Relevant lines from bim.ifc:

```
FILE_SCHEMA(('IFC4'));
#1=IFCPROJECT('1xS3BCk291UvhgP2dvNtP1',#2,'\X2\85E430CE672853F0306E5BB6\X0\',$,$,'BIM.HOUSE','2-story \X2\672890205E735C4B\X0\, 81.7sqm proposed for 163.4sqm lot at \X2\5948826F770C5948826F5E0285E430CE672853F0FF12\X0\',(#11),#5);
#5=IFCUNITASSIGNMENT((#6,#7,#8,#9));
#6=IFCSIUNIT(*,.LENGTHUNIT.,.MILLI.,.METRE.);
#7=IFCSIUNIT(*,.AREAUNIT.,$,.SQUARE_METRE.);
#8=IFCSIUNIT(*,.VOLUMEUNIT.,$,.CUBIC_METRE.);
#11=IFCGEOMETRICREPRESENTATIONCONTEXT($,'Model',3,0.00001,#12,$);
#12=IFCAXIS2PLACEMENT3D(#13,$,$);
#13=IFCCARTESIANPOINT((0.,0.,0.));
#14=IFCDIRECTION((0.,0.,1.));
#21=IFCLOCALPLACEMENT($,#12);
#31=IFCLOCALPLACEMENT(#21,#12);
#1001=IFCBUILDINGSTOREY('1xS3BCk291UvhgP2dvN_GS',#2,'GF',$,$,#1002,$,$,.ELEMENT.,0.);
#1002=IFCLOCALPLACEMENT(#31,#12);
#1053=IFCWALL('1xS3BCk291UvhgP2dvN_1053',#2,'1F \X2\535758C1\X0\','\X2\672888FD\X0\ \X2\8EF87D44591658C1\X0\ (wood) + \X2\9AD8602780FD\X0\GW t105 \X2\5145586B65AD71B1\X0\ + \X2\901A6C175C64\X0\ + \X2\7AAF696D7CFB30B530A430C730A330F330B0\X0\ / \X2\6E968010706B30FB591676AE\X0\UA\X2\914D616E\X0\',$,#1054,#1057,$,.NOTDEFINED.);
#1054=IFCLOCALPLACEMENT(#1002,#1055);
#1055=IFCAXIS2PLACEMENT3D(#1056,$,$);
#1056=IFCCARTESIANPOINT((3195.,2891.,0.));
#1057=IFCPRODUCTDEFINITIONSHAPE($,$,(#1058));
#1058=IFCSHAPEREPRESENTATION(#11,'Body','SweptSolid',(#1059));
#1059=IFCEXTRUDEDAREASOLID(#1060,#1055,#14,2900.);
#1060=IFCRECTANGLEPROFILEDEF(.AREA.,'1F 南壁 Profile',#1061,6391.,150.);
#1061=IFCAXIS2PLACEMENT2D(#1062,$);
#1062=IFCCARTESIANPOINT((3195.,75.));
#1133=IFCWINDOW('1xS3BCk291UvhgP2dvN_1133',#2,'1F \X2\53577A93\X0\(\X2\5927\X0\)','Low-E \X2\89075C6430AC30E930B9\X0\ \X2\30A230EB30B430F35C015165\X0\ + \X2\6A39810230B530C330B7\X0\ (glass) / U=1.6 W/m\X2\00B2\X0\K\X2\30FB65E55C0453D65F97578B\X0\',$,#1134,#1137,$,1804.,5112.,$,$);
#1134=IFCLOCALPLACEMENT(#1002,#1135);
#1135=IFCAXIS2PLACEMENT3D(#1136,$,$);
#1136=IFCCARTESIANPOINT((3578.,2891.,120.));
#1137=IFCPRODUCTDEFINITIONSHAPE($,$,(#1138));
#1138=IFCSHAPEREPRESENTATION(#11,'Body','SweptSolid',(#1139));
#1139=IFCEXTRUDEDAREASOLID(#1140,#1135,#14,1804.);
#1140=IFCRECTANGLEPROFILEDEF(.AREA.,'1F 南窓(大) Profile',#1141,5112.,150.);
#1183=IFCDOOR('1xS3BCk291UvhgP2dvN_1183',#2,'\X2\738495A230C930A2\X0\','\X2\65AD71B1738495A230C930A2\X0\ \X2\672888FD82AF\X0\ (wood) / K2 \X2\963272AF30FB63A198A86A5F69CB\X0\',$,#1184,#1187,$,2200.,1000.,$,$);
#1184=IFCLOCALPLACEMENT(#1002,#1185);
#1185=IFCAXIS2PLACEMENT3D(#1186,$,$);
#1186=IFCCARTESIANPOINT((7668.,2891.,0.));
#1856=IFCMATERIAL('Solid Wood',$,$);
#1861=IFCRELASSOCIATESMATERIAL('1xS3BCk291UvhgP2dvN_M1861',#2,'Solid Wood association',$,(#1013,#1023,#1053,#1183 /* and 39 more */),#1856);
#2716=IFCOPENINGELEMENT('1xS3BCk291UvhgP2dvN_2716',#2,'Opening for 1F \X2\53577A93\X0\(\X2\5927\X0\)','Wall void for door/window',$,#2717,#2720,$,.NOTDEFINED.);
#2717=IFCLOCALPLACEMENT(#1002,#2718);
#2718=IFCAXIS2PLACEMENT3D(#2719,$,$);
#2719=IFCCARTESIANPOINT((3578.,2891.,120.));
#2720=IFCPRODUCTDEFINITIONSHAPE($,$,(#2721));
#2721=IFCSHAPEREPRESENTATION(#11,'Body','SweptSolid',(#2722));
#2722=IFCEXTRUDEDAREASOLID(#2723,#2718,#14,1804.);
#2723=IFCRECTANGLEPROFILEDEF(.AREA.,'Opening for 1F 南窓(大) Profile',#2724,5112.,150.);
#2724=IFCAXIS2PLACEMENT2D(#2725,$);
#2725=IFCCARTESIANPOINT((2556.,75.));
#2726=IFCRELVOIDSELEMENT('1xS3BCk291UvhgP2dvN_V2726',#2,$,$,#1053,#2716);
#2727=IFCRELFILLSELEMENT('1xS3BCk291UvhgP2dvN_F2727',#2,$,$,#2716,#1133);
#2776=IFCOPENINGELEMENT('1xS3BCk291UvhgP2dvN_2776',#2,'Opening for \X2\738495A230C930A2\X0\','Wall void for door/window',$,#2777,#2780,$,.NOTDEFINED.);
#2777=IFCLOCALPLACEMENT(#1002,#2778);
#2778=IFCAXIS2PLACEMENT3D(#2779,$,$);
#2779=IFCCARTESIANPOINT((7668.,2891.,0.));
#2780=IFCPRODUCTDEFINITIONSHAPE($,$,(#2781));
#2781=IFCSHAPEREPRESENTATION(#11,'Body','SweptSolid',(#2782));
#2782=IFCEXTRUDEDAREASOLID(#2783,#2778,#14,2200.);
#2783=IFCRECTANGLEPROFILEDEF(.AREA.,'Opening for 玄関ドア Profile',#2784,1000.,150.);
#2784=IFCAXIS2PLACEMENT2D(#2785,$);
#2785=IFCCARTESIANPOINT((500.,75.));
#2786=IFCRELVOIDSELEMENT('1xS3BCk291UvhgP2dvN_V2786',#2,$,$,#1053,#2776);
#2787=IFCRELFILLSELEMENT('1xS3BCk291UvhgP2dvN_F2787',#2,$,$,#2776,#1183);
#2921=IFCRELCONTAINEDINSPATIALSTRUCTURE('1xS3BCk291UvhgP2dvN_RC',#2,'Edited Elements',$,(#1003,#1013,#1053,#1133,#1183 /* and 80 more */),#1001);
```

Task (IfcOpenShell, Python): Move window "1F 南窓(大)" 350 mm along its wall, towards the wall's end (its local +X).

```python
import ifcopenshell
import ifcopenshell.api.geometry
import ifcopenshell.util.placement
import ifcopenshell.util.unit

model = ifcopenshell.open("bim.ifc")
unit_scale = ifcopenshell.util.unit.calculate_unit_scale(model)

window = model.by_guid("1xS3BCk291UvhgP2dvN_1133")
opening = window.FillsVoids[0].RelatingOpeningElement
wall = opening.VoidsElements[0].RelatingBuildingElement

wall_matrix = ifcopenshell.util.placement.get_local_placement(wall.ObjectPlacement)
shift = wall_matrix[:3, 0] * 0.35 / unit_scale
before = ifcopenshell.util.placement.get_local_placement(window.ObjectPlacement)[:3, 3].copy()

# The window is not placed relative to its opening, so move both.
for product in (opening, window):
    matrix = ifcopenshell.util.placement.get_local_placement(product.ObjectPlacement)
    matrix[:3, 3] += shift
    ifcopenshell.api.geometry.edit_object_placement(model, product=product, matrix=matrix, is_si=False)

after = ifcopenshell.util.placement.get_local_placement(window.ObjectPlacement)[:3, 3]
print("window moved by", (after - before).round(3) + 0.0)

model.write("bim_rev.ifc")
```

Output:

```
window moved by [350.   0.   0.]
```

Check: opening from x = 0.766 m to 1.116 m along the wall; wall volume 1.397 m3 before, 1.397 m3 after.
